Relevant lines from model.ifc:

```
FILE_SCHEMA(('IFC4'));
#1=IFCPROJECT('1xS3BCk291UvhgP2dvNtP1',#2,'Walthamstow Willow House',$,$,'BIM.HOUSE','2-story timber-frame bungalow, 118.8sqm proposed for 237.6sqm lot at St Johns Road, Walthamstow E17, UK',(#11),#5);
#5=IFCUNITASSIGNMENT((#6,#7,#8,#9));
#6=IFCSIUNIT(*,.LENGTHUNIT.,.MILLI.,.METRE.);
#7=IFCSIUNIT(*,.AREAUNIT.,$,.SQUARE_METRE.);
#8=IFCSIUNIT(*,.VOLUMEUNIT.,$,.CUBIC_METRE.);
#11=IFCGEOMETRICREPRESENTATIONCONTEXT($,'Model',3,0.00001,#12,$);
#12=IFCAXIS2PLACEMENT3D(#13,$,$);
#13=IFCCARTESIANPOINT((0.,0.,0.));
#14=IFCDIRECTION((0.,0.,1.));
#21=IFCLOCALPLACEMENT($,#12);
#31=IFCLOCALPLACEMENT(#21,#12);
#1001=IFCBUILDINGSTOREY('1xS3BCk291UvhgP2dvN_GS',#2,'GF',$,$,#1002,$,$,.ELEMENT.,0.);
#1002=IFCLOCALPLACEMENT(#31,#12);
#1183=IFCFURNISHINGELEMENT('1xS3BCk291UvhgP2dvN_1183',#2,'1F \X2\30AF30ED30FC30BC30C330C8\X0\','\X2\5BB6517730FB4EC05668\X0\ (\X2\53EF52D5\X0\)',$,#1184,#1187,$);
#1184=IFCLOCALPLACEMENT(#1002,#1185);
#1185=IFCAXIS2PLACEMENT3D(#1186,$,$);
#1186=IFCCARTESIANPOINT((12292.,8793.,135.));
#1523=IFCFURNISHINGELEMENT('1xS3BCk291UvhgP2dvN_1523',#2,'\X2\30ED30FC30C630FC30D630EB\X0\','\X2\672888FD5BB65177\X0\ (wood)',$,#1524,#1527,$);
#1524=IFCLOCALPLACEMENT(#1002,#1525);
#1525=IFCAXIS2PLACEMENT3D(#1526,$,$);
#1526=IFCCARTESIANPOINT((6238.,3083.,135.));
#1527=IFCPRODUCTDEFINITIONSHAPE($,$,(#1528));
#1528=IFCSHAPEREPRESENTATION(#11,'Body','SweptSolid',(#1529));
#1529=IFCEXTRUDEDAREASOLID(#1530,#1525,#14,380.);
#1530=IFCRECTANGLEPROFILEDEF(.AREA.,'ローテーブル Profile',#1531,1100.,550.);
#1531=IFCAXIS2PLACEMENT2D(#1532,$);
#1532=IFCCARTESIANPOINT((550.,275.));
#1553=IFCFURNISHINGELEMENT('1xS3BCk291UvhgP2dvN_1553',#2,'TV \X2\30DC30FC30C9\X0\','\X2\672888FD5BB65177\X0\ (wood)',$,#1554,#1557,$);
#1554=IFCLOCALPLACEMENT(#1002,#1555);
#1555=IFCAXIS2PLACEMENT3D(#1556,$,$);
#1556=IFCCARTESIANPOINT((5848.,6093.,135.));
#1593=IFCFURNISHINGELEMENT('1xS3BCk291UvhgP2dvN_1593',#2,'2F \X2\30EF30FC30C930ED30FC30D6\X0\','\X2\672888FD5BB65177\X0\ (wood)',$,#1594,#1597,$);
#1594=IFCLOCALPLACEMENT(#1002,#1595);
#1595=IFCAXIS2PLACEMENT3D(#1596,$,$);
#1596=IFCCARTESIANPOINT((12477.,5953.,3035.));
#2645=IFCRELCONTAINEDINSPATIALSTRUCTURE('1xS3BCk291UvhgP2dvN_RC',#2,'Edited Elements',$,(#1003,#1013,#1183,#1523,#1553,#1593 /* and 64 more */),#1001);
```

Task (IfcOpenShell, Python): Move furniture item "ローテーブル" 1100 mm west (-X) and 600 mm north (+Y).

```python
import ifcopenshell
import ifcopenshell.api.geometry
import ifcopenshell.util.placement
import ifcopenshell.util.unit

model = ifcopenshell.open("model.ifc")
unit_scale = ifcopenshell.util.unit.calculate_unit_scale(model)

item = model.by_guid("1xS3BCk291UvhgP2dvN_1523")
matrix = ifcopenshell.util.placement.get_local_placement(item.ObjectPlacement)
matrix[0, 3] -= 1.1 / unit_scale
matrix[1, 3] += 0.6 / unit_scale
ifcopenshell.api.geometry.edit_object_placement(model, product=item, matrix=matrix, is_si=False)

print(ifcopenshell.util.placement.get_local_placement(item.ObjectPlacement).round(3) + 0.0)

model.write("model_rev.ifc")
```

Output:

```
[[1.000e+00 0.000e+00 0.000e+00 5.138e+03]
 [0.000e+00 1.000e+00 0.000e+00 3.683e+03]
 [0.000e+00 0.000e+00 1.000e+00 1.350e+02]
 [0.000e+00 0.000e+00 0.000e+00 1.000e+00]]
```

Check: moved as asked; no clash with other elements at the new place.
